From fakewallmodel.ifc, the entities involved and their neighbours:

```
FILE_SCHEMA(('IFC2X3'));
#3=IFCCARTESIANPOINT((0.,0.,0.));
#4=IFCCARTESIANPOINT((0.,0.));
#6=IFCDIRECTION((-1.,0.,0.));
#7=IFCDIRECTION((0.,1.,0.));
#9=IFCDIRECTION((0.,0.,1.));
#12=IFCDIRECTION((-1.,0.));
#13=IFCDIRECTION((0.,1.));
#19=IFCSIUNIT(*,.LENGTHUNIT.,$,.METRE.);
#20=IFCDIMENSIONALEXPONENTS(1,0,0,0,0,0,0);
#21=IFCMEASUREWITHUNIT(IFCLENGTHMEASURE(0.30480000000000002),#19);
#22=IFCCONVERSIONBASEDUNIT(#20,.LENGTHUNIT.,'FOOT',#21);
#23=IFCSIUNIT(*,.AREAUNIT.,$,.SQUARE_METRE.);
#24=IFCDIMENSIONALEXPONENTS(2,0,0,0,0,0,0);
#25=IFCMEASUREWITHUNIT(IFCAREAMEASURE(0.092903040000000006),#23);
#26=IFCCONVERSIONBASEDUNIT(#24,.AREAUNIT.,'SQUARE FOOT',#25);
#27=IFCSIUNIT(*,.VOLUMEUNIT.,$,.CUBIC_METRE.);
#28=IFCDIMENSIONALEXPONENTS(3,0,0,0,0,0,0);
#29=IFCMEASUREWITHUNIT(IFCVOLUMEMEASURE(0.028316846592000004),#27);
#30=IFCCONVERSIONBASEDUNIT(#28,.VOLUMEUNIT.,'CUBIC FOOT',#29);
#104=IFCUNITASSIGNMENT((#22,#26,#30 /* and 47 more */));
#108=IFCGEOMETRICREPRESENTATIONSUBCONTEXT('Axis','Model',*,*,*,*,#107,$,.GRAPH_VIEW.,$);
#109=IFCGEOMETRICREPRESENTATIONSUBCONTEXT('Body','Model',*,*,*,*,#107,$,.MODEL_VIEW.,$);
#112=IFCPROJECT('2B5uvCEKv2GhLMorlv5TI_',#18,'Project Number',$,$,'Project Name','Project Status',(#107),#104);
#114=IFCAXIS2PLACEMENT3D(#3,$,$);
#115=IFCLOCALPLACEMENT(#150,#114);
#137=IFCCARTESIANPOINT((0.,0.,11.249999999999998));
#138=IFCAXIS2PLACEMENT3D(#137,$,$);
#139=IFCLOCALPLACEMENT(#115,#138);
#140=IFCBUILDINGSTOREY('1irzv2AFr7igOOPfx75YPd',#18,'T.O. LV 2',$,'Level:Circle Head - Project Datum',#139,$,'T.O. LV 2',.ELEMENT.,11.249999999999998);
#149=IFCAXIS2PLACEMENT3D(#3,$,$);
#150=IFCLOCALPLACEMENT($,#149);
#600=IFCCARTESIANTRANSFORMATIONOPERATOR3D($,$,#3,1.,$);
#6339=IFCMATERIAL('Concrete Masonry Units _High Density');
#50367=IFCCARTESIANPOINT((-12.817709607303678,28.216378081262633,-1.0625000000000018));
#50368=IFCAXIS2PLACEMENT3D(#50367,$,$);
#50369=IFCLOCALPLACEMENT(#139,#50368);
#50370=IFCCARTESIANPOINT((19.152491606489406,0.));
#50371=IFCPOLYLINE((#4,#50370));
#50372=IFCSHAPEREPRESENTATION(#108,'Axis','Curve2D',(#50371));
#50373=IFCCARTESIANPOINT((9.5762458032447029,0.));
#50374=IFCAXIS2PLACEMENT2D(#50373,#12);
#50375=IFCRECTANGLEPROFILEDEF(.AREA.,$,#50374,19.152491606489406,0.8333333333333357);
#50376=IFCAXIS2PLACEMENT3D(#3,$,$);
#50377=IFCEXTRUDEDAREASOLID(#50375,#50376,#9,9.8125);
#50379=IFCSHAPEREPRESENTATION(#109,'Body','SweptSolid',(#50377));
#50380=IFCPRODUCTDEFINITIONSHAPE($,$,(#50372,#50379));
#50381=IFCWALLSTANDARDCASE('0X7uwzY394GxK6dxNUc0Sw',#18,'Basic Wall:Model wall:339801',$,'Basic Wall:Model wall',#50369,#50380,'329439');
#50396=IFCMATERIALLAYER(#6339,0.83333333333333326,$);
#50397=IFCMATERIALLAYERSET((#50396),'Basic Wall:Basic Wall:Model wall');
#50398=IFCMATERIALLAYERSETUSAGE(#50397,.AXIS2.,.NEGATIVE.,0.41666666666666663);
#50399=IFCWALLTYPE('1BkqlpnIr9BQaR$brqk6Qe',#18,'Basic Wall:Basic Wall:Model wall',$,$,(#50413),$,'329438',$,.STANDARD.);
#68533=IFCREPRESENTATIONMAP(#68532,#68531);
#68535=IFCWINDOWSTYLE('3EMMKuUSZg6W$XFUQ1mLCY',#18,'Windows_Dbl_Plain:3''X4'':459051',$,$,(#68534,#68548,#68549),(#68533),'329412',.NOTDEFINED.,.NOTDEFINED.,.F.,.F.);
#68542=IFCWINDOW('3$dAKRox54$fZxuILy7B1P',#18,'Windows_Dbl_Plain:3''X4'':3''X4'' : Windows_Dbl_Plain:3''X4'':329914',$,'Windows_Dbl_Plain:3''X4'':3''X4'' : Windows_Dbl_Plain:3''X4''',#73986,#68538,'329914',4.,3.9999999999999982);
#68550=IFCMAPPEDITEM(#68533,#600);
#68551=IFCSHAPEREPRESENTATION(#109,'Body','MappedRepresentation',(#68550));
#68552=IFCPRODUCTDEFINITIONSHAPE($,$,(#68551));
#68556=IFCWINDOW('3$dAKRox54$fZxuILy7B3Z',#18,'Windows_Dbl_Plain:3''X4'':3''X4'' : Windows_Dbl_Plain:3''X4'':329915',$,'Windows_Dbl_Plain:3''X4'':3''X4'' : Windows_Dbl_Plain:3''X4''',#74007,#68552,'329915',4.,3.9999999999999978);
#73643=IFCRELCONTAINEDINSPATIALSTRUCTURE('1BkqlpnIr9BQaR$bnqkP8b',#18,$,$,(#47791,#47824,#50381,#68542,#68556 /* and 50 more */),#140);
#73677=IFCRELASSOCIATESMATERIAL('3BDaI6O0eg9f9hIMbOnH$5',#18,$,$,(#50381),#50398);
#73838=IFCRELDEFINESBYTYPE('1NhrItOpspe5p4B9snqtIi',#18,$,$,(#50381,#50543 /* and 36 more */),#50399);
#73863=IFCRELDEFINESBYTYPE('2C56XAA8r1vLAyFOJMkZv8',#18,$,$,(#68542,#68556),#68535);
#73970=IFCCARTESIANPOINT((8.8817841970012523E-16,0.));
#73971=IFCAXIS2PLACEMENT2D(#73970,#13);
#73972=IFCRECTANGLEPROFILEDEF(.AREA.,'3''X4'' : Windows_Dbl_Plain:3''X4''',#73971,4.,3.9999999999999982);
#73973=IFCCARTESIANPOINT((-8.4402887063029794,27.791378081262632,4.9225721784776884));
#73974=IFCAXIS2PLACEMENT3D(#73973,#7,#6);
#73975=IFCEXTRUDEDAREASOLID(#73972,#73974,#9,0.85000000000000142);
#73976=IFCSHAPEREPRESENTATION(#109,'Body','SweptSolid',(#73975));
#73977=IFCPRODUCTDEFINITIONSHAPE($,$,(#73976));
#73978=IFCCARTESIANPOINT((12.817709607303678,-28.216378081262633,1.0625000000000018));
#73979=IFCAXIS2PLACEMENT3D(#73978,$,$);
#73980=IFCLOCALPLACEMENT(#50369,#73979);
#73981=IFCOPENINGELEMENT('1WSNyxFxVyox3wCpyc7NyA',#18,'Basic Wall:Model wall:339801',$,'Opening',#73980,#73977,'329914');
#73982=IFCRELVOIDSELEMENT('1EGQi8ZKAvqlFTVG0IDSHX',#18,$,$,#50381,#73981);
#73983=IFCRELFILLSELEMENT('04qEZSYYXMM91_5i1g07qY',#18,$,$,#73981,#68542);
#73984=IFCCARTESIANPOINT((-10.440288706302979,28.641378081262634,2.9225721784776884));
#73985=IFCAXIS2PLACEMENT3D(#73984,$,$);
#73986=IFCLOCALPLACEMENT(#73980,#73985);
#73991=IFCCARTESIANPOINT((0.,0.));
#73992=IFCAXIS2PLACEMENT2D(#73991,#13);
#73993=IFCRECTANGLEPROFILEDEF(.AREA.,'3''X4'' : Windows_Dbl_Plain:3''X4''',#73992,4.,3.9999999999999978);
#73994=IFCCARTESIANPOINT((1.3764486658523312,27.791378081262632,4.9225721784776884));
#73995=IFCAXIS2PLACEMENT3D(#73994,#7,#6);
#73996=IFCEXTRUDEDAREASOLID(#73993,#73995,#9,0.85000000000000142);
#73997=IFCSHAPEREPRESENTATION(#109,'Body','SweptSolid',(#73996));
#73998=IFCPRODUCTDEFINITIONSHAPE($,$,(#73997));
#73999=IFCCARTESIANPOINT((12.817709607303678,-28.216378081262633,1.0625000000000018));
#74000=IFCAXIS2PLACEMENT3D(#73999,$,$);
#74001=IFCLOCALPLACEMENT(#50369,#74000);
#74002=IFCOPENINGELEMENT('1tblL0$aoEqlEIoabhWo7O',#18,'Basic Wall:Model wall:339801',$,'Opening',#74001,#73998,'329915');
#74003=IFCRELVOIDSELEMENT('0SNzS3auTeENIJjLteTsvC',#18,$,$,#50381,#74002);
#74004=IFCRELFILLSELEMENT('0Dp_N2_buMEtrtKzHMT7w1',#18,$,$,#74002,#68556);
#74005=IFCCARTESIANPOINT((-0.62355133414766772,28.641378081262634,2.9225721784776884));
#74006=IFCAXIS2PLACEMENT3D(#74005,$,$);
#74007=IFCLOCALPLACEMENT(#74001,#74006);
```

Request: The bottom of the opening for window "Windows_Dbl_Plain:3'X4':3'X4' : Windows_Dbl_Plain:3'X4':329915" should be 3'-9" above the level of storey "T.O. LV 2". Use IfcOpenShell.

```python
import numpy as np
import ifcopenshell
import ifcopenshell.api.geometry
import ifcopenshell.geom
import ifcopenshell.util.element
import ifcopenshell.util.placement
import ifcopenshell.util.shape
import ifcopenshell.util.unit

model = ifcopenshell.open("fakewallmodel.ifc")
unit_scale = ifcopenshell.util.unit.calculate_unit_scale(model)

window = model.by_guid("3$dAKRox54$fZxuILy7B3Z")
opening = window.FillsVoids[0].RelatingOpeningElement
storey = ifcopenshell.util.element.get_container(window, ifc_class="IfcBuildingStorey")
level = ifcopenshell.util.placement.get_local_placement(storey.ObjectPlacement)[2, 3]

# The opening's origin need not be at the sill, so measure its lowest point.
shape = ifcopenshell.geom.create_shape(ifcopenshell.geom.settings(), opening)
bottom = ifcopenshell.util.shape.get_shape_bottom_elevation(shape, shape.geometry) / unit_scale
dz = level + 45 * 0.0254 / unit_scale - bottom

shift = np.array([0.0, 0.0, dz])
# The window is placed relative to its opening, so it follows when the opening moves.
matrix = ifcopenshell.util.placement.get_local_placement(opening.ObjectPlacement)
matrix[:3, 3] += shift
ifcopenshell.api.geometry.edit_object_placement(
    model, product=opening, matrix=matrix, is_si=False, should_transform_children=True
)

print(f"moved by {dz * unit_scale:+.3f} m")

model.write("fakewallmodel_updated.ifc")
```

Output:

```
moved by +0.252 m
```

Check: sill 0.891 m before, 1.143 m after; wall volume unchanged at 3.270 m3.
